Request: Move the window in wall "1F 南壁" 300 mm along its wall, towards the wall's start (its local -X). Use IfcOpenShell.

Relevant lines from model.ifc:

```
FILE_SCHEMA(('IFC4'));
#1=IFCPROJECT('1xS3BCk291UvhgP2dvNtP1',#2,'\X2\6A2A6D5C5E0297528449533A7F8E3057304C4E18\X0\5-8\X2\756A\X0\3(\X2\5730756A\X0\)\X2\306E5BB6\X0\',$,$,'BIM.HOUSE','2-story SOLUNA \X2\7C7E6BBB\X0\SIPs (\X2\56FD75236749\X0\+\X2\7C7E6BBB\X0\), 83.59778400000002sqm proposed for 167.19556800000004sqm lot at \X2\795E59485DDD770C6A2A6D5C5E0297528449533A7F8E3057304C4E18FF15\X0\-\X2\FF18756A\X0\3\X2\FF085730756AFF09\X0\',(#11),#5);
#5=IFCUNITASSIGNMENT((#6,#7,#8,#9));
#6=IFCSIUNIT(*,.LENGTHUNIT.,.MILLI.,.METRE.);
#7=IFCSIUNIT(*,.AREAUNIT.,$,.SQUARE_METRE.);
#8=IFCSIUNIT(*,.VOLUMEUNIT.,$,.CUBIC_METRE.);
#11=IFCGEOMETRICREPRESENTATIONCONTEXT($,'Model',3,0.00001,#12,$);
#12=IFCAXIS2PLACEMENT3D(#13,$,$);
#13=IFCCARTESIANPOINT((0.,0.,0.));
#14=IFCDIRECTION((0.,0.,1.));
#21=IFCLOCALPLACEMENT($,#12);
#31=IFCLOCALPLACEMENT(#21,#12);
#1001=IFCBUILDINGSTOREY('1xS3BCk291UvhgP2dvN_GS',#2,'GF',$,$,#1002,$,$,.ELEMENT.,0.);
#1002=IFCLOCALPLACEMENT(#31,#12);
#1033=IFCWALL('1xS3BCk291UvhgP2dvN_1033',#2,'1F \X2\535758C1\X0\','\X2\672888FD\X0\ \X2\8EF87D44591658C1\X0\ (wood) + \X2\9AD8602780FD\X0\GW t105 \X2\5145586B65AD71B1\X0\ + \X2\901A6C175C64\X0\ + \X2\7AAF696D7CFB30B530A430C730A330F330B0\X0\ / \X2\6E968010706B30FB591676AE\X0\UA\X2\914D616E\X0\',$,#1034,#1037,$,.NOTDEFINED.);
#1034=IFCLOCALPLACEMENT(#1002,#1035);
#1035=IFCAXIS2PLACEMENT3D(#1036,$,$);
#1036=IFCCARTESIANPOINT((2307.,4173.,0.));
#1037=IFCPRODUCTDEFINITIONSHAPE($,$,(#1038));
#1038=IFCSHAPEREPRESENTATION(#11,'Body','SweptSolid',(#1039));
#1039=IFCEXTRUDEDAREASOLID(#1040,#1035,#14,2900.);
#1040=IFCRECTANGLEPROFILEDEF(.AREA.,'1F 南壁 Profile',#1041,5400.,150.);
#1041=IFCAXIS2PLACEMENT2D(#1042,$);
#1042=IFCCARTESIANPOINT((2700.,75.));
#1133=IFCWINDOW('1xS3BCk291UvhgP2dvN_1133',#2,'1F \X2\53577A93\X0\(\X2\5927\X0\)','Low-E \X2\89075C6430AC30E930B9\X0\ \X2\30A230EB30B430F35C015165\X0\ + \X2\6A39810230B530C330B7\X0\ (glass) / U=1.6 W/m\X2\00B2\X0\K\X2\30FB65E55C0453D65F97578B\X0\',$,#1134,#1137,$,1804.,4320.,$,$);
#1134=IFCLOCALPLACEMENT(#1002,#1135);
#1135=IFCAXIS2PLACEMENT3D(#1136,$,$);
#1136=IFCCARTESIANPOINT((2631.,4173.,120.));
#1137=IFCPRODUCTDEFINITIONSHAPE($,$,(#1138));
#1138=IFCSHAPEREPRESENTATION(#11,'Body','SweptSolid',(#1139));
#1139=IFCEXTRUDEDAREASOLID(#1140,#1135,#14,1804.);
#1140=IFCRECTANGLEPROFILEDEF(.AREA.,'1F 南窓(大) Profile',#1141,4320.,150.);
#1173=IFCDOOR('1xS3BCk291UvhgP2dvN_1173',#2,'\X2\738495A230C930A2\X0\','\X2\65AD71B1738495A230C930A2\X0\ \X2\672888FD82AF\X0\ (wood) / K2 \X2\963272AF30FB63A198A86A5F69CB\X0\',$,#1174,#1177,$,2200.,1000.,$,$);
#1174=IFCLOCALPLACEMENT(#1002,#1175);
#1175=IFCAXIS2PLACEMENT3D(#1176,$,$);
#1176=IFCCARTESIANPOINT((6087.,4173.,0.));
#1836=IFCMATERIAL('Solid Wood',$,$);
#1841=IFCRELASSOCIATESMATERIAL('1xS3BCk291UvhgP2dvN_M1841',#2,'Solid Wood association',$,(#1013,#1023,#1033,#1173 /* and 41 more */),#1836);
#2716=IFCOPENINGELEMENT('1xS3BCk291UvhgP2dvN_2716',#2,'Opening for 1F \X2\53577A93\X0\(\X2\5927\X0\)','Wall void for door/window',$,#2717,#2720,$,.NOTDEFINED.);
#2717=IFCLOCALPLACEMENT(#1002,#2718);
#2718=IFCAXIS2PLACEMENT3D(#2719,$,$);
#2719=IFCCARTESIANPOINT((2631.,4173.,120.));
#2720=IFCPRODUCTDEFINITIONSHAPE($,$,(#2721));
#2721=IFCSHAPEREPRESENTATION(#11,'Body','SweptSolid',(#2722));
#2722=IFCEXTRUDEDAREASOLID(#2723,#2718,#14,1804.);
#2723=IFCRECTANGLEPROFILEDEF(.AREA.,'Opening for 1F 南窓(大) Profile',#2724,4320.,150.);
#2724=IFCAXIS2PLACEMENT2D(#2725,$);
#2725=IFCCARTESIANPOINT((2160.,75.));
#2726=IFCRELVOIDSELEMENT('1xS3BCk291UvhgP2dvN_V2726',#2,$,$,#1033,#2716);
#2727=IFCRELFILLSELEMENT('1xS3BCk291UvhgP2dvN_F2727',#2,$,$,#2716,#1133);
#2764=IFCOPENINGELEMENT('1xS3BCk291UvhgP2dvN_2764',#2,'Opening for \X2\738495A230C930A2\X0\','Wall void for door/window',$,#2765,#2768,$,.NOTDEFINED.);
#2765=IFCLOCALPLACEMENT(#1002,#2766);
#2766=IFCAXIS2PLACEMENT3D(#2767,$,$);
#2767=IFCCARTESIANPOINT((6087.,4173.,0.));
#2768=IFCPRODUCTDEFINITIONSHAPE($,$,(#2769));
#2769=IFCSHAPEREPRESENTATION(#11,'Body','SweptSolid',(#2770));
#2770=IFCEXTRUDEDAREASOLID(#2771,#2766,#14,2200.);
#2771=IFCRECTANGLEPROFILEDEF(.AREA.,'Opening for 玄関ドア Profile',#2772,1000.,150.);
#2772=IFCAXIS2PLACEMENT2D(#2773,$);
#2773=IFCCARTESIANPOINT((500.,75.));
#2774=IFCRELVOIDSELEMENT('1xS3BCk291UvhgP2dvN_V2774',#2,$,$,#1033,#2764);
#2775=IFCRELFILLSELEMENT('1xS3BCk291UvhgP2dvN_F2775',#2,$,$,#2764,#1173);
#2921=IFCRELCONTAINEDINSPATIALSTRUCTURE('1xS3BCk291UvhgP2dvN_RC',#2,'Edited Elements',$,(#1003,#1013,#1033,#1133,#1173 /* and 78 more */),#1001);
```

```python
import ifcopenshell
import ifcopenshell.api.geometry
import ifcopenshell.util.placement
import ifcopenshell.util.unit

model = ifcopenshell.open("model.ifc")
unit_scale = ifcopenshell.util.unit.calculate_unit_scale(model)

window = model.by_id(1133)
opening = window.FillsVoids[0].RelatingOpeningElement
wall = opening.VoidsElements[0].RelatingBuildingElement

wall_matrix = ifcopenshell.util.placement.get_local_placement(wall.ObjectPlacement)
shift = wall_matrix[:3, 0] * -0.3 / unit_scale
before = ifcopenshell.util.placement.get_local_placement(window.ObjectPlacement)[:3, 3].copy()

# The window is not placed relative to its opening, so move both.
for product in (opening, window):
    matrix = ifcopenshell.util.placement.get_local_placement(product.ObjectPlacement)
    matrix[:3, 3] += shift
    ifcopenshell.api.geometry.edit_object_placement(model, product=product, matrix=matrix, is_si=False)

after = ifcopenshell.util.placement.get_local_placement(window.ObjectPlacement)[:3, 3]
print("window moved by", (after - before).round(3) + 0.0)

model.write("model_updated.ifc")
```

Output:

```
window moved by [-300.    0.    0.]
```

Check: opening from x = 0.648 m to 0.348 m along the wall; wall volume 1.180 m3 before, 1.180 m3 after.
